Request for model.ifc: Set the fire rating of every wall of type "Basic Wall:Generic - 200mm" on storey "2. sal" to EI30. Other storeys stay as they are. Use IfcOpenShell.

First a look at what the model holds.

```python
import ifcopenshell
import ifcopenshell.util.element

model = ifcopenshell.open("model.ifc")
print(model.schema)
storey = next(s for s in model.by_type("IfcBuildingStorey") if s.Name == "2. sal")
walls = [e for e in ifcopenshell.util.element.get_decomposition(storey) if e.is_a("IfcWall")]
seen = {}
for e in walls:
    element_type = ifcopenshell.util.element.get_type(e)
    key = (element_type.Name if element_type != e and element_type else None, ifcopenshell.util.element.get_pset(e, "Pset_WallCommon", "FireRating"))
    seen[key] = seen.get(key, 0) + 1
for (name, value), count in sorted(seen.items(), key=str):
    print(count, "x", name, "|", value)
```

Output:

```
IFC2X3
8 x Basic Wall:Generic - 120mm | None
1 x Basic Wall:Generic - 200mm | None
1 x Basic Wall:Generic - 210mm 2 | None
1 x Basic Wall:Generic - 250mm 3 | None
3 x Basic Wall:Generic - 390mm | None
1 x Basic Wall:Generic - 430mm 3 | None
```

```python
import ifcopenshell
import ifcopenshell.api.pset
import ifcopenshell.util.element

model = ifcopenshell.open("model.ifc")

storey = next(s for s in model.by_type("IfcBuildingStorey") if s.Name == "2. sal")
walls = [e for e in ifcopenshell.util.element.get_decomposition(storey) if e.is_a("IfcWall")]

count = 0
for e in walls:
    element_type = ifcopenshell.util.element.get_type(e)
    if element_type in (None, e) or element_type.Name != "Basic Wall:Generic - 200mm":
        continue
    # add_pset returns the element's existing set when there is one.
    pset = ifcopenshell.api.pset.add_pset(model, product=e, name="Pset_WallCommon")
    ifcopenshell.api.pset.edit_pset(model, pset=pset, properties={"FireRating": "EI30"})
    count += 1

print(count, "walls updated")

model.write("model_updated.ifc")
```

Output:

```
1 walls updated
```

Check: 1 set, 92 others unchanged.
